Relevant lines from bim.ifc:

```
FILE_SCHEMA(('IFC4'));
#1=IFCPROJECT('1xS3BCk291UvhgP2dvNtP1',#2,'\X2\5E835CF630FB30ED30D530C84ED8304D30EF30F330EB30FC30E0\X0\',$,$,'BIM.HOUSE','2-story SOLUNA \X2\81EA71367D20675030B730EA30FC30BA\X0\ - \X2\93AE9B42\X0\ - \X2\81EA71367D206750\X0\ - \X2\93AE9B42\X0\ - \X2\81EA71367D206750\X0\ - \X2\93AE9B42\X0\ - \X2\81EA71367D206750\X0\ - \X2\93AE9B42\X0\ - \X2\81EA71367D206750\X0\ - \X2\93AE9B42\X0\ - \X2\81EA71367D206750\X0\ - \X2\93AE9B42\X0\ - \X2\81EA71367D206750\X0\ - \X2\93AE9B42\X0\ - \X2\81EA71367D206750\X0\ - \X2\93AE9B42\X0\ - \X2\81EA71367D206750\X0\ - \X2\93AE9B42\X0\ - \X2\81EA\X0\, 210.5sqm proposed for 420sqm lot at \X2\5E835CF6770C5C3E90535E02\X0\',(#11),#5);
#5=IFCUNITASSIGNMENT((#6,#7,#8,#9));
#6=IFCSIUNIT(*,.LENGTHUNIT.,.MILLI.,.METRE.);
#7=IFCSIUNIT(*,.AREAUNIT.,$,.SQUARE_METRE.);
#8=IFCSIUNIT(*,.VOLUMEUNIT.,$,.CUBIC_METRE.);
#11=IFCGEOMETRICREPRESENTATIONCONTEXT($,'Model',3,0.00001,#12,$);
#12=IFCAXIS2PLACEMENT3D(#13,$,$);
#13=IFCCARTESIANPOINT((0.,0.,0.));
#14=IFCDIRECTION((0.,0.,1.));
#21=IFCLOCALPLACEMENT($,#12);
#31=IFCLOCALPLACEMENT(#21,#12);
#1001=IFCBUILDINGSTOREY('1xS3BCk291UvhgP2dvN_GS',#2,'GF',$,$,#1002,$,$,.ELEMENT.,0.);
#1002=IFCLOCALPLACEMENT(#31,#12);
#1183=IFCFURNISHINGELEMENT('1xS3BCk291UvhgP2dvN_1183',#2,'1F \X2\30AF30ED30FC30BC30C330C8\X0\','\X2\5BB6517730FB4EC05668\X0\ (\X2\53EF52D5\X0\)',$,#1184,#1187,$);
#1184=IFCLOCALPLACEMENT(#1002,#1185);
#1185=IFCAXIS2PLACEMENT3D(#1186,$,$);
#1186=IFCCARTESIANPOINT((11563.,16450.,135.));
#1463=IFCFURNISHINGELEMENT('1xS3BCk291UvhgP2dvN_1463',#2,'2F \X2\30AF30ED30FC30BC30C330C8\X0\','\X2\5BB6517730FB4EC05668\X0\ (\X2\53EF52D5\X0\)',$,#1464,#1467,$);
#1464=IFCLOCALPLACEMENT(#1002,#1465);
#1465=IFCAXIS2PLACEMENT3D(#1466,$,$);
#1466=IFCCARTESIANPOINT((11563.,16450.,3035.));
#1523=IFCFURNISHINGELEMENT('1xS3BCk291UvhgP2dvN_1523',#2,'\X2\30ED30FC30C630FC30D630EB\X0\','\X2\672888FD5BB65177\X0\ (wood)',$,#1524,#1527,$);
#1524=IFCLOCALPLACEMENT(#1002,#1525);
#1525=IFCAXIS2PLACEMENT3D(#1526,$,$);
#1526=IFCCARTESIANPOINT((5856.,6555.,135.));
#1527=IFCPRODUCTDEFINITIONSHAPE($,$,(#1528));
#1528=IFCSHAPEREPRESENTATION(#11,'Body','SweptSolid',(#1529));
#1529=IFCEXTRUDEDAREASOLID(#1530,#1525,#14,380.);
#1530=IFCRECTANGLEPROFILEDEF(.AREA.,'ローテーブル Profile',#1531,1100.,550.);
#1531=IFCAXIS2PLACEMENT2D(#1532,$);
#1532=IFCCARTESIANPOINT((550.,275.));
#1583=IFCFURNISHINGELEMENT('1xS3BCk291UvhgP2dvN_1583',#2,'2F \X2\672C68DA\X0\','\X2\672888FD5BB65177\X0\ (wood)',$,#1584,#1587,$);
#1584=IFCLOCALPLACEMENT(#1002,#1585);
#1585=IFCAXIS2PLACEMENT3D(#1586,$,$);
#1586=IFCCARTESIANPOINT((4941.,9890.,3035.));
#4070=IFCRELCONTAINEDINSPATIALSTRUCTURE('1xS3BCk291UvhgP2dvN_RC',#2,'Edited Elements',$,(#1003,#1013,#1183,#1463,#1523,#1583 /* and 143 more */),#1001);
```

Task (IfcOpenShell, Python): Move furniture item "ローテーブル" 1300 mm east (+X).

```python
import ifcopenshell
import ifcopenshell.api.geometry
import ifcopenshell.util.placement
import ifcopenshell.util.unit

model = ifcopenshell.open("bim.ifc")
unit_scale = ifcopenshell.util.unit.calculate_unit_scale(model)

item = model.by_guid("1xS3BCk291UvhgP2dvN_1523")
matrix = ifcopenshell.util.placement.get_local_placement(item.ObjectPlacement)
matrix[0, 3] += 1.3 / unit_scale
ifcopenshell.api.geometry.edit_object_placement(model, product=item, matrix=matrix, is_si=False)

print(ifcopenshell.util.placement.get_local_placement(item.ObjectPlacement).round(3) + 0.0)

model.write("bim_updated.ifc")
```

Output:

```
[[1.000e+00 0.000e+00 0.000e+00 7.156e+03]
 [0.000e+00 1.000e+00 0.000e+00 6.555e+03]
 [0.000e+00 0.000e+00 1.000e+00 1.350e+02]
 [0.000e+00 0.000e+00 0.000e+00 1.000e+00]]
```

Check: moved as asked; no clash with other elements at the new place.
